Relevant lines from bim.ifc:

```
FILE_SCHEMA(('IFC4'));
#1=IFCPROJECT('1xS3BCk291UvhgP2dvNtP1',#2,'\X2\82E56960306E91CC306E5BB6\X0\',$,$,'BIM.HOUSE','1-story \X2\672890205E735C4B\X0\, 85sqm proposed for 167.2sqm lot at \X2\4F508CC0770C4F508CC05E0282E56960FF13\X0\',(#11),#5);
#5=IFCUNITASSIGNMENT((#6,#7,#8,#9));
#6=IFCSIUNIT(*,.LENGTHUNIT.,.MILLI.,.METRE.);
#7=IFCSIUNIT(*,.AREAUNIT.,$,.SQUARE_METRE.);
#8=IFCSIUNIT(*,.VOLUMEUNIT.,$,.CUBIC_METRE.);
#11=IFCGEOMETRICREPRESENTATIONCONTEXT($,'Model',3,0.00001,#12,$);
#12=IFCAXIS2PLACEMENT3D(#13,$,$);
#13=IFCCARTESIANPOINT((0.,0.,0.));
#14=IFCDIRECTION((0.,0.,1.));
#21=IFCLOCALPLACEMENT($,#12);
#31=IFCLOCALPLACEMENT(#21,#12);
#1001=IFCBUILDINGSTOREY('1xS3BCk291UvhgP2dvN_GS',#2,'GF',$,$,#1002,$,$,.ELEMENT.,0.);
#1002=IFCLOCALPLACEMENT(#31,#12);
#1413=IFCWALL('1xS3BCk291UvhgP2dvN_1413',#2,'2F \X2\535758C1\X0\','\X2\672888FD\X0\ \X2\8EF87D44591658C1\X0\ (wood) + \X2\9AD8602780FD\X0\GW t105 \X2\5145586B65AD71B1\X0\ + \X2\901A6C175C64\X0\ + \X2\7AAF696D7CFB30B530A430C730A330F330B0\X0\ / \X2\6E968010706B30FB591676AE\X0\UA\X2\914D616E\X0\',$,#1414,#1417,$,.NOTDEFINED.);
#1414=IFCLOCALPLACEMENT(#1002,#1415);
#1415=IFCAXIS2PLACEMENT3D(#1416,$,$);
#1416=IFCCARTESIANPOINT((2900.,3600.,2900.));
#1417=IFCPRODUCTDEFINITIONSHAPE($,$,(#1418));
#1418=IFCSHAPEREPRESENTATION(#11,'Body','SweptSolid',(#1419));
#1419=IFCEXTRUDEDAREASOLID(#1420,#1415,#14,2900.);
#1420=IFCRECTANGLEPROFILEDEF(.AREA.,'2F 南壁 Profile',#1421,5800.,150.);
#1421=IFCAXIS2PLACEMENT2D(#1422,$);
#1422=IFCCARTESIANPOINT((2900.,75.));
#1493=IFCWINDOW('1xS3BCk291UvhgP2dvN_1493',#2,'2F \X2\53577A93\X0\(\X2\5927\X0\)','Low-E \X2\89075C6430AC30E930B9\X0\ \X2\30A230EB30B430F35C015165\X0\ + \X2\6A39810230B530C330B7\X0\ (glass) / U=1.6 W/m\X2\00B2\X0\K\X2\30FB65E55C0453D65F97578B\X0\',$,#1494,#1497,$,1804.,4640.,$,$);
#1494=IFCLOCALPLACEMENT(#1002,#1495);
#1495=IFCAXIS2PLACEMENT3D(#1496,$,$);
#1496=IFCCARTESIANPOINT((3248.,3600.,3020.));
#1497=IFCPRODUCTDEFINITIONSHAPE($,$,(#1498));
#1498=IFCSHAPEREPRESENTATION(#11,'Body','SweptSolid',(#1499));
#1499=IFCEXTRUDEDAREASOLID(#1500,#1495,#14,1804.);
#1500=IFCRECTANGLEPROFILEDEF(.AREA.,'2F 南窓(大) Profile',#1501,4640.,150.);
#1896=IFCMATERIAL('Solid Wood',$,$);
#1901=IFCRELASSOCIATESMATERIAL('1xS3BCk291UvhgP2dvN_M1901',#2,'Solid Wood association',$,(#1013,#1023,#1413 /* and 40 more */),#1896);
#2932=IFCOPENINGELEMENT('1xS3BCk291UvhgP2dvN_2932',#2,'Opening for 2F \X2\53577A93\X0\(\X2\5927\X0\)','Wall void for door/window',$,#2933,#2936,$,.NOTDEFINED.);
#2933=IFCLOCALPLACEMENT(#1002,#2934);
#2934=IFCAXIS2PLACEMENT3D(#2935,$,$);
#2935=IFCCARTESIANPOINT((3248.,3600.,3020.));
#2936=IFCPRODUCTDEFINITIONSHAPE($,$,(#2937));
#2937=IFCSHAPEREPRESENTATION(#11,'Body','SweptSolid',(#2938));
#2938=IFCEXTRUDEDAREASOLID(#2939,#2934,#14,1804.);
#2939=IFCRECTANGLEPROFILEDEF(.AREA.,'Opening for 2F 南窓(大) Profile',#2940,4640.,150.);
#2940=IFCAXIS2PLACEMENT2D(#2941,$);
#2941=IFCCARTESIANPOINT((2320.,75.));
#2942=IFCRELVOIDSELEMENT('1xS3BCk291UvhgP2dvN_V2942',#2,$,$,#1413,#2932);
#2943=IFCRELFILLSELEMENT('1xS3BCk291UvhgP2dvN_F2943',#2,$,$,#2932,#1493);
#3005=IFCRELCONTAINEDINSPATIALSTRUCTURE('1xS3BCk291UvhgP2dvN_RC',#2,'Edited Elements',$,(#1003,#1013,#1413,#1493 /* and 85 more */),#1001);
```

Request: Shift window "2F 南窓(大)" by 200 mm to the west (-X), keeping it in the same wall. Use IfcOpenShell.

```python
import ifcopenshell
import ifcopenshell.api.geometry
import ifcopenshell.util.placement

model = ifcopenshell.open("bim.ifc")

window = model.by_id(1493)
opening = window.FillsVoids[0].RelatingOpeningElement
wall = opening.VoidsElements[0].RelatingBuildingElement

wall_matrix = ifcopenshell.util.placement.get_local_placement(wall.ObjectPlacement)
shift = wall_matrix[:3, 0] * -200.0
before = ifcopenshell.util.placement.get_local_placement(window.ObjectPlacement)[:3, 3].copy()

# The window is not placed relative to its opening, so move both.
for product in (opening, window):
    matrix = ifcopenshell.util.placement.get_local_placement(product.ObjectPlacement)
    matrix[:3, 3] += shift
    ifcopenshell.api.geometry.edit_object_placement(model, product=product, matrix=matrix, is_si=False)

after = ifcopenshell.util.placement.get_local_placement(window.ObjectPlacement)[:3, 3]
print("window moved by", (after - before).round(3) + 0.0)

model.write("bim_rev.ifc")
```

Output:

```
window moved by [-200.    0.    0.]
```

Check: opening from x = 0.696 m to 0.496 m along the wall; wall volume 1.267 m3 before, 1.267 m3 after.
